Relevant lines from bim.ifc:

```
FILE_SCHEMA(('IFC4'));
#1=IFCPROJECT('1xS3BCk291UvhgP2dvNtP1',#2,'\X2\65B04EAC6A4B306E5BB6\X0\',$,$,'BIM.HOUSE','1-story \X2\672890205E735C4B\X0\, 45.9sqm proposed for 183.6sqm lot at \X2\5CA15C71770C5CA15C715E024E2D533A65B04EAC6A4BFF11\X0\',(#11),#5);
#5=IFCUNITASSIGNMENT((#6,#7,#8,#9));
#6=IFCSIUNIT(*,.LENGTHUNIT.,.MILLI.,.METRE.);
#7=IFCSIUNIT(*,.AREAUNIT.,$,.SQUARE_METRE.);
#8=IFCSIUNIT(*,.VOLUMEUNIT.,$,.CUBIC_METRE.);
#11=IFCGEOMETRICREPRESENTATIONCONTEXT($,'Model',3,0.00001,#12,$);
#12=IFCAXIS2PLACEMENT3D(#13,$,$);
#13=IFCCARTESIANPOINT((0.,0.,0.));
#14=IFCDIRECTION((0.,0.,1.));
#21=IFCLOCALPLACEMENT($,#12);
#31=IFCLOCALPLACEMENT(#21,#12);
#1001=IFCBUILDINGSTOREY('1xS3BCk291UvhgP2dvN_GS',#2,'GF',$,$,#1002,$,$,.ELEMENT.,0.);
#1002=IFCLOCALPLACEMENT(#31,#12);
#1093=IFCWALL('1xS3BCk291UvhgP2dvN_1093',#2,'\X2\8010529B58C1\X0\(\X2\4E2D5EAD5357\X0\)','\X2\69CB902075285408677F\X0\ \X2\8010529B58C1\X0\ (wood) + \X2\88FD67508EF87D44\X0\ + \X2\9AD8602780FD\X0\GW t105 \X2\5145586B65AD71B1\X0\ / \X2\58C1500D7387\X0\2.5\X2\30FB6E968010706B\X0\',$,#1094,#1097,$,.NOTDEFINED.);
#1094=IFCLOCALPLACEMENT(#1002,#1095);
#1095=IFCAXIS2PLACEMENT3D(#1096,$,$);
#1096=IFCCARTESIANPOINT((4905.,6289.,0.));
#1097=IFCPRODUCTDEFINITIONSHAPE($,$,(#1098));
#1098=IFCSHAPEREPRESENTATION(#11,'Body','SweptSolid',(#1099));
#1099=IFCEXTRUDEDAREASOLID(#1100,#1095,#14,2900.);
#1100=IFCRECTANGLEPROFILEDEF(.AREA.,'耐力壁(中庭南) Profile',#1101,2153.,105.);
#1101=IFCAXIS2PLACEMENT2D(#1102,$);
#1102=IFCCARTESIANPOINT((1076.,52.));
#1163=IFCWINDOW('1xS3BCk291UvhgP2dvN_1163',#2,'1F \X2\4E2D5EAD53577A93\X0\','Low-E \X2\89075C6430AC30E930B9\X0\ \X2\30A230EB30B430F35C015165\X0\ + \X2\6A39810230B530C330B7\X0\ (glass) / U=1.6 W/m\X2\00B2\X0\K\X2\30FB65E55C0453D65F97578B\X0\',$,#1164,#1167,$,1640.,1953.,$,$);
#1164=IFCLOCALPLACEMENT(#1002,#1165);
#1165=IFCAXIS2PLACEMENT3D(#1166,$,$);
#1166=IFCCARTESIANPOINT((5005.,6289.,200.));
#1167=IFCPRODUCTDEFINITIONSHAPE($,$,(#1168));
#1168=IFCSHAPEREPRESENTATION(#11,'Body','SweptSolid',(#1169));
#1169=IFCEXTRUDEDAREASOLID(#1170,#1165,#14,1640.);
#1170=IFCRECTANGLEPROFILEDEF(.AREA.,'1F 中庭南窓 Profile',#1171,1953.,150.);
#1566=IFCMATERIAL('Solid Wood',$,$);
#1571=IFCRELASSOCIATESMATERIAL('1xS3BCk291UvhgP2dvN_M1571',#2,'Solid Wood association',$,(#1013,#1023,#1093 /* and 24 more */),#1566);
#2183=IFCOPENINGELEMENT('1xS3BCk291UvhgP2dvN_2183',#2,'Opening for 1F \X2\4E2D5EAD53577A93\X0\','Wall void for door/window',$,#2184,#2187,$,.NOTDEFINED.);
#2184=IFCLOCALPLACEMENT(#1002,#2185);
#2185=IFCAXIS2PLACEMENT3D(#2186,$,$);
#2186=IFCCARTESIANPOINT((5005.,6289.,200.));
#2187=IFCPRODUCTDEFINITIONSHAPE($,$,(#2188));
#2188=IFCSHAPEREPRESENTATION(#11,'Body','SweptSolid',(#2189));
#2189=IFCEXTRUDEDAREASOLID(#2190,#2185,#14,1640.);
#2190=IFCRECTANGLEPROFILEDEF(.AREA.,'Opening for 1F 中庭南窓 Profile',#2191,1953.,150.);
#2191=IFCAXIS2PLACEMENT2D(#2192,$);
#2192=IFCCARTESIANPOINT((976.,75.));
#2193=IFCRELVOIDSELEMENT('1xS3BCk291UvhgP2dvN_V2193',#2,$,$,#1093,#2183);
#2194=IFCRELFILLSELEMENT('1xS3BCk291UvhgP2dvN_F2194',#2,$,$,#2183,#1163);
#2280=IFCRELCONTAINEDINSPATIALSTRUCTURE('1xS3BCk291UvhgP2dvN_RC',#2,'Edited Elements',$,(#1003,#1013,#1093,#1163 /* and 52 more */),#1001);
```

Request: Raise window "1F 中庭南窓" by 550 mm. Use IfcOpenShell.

```python
import numpy as np
import ifcopenshell
import ifcopenshell.api.geometry
import ifcopenshell.util.placement
import ifcopenshell.util.unit

model = ifcopenshell.open("bim.ifc")
unit_scale = ifcopenshell.util.unit.calculate_unit_scale(model)

window = model.by_guid("1xS3BCk291UvhgP2dvN_1163")
opening = window.FillsVoids[0].RelatingOpeningElement
dz = 550.0

shift = np.array([0.0, 0.0, dz])
# The window is not placed relative to its opening, so move both.
for product in (opening, window):
    matrix = ifcopenshell.util.placement.get_local_placement(product.ObjectPlacement)
    matrix[:3, 3] += shift
    ifcopenshell.api.geometry.edit_object_placement(model, product=product, matrix=matrix, is_si=False)

print(f"moved by {dz * unit_scale:+.3f} m")

model.write("bim_rev.ifc")
```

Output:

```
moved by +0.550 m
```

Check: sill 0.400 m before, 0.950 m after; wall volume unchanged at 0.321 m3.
